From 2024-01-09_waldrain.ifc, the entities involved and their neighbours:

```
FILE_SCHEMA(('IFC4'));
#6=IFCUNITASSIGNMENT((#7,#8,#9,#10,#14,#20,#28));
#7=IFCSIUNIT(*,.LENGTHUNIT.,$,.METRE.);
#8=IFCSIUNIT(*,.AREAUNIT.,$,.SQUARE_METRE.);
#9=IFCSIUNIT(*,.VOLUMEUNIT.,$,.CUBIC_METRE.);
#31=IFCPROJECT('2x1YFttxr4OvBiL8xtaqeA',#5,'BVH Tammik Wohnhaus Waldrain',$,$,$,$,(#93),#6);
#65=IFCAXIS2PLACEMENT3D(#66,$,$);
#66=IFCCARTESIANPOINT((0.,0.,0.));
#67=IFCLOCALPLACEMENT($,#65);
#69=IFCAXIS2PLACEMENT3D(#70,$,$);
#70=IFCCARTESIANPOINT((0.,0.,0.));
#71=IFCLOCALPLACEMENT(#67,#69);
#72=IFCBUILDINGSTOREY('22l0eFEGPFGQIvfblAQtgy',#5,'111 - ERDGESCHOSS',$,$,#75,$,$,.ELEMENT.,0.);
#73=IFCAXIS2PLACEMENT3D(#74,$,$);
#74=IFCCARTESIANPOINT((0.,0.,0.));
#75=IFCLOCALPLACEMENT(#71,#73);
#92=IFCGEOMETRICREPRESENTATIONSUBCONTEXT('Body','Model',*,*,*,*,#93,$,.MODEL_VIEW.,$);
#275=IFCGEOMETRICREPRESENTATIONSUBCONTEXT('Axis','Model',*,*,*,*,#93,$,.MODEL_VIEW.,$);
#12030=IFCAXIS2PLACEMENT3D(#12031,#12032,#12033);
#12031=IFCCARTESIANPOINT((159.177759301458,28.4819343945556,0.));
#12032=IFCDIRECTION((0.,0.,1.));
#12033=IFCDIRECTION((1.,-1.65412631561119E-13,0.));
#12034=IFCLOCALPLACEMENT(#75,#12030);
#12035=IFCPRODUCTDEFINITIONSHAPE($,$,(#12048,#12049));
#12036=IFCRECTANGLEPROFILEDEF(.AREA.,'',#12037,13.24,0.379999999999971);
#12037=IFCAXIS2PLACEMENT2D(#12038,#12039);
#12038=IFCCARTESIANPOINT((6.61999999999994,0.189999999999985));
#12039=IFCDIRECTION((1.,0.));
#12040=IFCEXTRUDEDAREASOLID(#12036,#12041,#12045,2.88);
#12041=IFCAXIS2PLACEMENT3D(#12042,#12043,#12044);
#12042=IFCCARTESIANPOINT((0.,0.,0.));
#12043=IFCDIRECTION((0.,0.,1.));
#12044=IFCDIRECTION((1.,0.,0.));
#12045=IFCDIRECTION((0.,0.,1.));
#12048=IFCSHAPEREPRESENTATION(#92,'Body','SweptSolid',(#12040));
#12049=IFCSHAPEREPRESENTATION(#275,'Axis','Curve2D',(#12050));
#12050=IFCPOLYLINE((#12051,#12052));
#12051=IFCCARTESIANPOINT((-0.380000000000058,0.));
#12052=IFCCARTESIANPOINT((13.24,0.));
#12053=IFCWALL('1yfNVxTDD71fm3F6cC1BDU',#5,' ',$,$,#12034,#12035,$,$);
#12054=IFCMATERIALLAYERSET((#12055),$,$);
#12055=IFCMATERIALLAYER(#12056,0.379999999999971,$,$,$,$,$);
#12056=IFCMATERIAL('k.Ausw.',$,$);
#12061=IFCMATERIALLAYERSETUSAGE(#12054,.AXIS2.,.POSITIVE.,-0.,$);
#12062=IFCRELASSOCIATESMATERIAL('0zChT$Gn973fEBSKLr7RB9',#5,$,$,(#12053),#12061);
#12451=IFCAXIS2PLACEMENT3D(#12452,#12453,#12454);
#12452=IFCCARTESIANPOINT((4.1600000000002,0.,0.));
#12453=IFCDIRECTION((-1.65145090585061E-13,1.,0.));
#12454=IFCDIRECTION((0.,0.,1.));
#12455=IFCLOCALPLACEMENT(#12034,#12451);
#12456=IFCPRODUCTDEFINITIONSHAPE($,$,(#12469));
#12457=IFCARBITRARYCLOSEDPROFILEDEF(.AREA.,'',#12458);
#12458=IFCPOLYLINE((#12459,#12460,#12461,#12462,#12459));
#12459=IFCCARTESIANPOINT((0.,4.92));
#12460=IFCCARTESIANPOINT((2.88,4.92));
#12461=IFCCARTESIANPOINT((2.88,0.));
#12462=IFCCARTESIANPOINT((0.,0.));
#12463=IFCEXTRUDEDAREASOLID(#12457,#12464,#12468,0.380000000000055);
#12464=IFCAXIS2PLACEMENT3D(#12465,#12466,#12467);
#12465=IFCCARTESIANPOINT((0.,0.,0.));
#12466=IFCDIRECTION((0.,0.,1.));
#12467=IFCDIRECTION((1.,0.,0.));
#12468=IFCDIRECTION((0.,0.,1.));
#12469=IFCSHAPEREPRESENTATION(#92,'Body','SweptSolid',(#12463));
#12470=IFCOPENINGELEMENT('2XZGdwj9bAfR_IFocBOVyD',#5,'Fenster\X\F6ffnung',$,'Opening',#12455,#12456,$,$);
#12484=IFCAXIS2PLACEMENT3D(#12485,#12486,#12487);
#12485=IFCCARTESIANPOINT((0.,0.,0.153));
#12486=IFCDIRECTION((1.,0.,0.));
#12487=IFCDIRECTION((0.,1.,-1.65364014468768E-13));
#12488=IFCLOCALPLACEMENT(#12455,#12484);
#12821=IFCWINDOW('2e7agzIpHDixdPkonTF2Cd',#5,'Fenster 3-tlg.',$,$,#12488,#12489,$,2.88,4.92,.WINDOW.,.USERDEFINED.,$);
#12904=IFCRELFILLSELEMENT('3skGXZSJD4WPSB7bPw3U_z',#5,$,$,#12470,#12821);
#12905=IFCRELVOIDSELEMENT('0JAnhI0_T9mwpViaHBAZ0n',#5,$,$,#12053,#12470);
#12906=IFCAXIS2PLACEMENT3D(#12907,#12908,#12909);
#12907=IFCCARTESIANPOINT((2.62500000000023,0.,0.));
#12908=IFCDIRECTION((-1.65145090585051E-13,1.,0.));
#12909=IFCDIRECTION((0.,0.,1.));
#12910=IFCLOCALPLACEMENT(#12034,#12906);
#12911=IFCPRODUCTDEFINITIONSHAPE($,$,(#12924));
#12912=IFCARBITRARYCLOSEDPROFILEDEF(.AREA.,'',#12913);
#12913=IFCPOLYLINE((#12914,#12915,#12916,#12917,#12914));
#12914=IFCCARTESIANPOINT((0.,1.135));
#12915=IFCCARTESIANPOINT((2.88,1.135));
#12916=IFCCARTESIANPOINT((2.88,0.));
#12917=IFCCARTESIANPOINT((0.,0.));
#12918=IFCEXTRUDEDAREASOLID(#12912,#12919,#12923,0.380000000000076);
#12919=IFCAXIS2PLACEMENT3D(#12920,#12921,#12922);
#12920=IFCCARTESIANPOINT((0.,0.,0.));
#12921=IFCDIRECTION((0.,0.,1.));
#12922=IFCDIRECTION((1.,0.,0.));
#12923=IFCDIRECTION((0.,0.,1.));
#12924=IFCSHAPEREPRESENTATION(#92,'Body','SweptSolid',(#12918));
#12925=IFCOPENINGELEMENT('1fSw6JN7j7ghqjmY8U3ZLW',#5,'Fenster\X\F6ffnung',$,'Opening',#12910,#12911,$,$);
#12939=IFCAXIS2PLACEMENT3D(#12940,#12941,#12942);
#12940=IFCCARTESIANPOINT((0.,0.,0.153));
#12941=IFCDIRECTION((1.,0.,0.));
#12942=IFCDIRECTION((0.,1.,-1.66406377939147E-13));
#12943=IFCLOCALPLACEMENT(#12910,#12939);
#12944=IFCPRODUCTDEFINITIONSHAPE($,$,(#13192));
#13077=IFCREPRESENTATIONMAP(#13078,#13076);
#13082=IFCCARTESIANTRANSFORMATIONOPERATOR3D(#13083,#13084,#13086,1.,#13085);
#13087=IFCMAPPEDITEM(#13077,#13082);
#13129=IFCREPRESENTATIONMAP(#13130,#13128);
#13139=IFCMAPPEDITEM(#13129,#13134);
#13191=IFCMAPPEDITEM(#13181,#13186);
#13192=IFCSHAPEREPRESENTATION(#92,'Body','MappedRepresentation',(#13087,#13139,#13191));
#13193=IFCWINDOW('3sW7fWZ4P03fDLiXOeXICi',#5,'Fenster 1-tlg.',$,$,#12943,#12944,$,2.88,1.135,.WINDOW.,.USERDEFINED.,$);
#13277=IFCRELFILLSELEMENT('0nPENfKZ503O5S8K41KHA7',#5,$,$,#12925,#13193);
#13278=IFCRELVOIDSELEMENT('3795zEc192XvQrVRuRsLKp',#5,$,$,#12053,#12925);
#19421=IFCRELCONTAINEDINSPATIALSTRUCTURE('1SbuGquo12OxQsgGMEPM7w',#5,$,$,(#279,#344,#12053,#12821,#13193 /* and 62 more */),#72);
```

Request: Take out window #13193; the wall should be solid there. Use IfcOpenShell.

```python
import ifcopenshell
import ifcopenshell.api.feature
import ifcopenshell.api.root
import ifcopenshell.geom
import ifcopenshell.util.shape

model = ifcopenshell.open("2024-01-09_waldrain.ifc")
settings = ifcopenshell.geom.settings()


def volume(element):
    """Net volume in cubic metres, openings subtracted."""
    shape = ifcopenshell.geom.create_shape(settings, element)
    return ifcopenshell.util.shape.get_volume(shape.geometry)


window = model.by_guid("3sW7fWZ4P03fDLiXOeXICi")
opening = window.FillsVoids[0].RelatingOpeningElement
wall = opening.VoidsElements[0].RelatingBuildingElement
before = volume(wall)

ifcopenshell.api.root.remove_product(model, product=window)
ifcopenshell.api.feature.remove_feature(model, feature=opening)

after = volume(wall)

print(f"wall volume {before:.3f} -> {after:.3f} m3")

model.write("2024-01-09_waldrain_v2.ifc")
```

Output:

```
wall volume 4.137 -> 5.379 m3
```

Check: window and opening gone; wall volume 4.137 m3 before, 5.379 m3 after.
